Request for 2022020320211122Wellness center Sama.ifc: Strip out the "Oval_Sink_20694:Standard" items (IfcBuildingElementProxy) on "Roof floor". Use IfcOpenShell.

First a look at what the model holds.

```python
import ifcopenshell
import ifcopenshell.util.element

model = ifcopenshell.open("2022020320211122Wellness center Sama.ifc")
print(model.schema)
storey = next(s for s in model.by_type("IfcBuildingStorey") if s.Name == "Roof floor")
proxies = [e for e in ifcopenshell.util.element.get_decomposition(storey) if e.is_a("IfcBuildingElementProxy")]
seen = {}
for e in proxies:
    element_type = ifcopenshell.util.element.get_type(e)
    name = element_type.Name if element_type not in (None, e) else None
    seen[name] = seen.get(name, 0) + 1
for name, count in sorted(seen.items(), key=str):
    print(count, "x", name)
```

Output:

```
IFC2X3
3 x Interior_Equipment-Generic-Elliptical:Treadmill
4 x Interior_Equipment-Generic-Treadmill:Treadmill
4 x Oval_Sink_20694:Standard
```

```python
import ifcopenshell
import ifcopenshell.api.root
import ifcopenshell.util.element

model = ifcopenshell.open("2022020320211122Wellness center Sama.ifc")

storey = next(s for s in model.by_type("IfcBuildingStorey") if s.Name == "Roof floor")
proxies = [e for e in ifcopenshell.util.element.get_decomposition(storey) if e.is_a("IfcBuildingElementProxy")]
targets = [e for e in proxies if (t := ifcopenshell.util.element.get_type(e)) not in (None, e) and t.Name == "Oval_Sink_20694:Standard"]

for e in targets:
    ifcopenshell.api.root.remove_product(model, product=e)
print(len(targets), "removed")

model.write("2022020320211122Wellness center Sama_updated.ifc")
```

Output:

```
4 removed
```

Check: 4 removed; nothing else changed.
